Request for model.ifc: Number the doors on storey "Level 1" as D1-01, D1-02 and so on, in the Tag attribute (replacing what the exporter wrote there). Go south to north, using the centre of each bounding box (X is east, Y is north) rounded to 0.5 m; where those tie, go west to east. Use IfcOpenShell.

First a look at what the model holds.

```python
import ifcopenshell
import ifcopenshell.util.element
import ifcopenshell.util.placement

model = ifcopenshell.open("model.ifc")
print(model.schema)
storey = next(s for s in model.by_type("IfcBuildingStorey") if s.Name == "Level 1")
doors = [e for e in ifcopenshell.util.element.get_decomposition(storey) if e.is_a("IfcDoor")]
for e in sorted(doors, key=lambda e: e.id()):
    origin = ifcopenshell.util.placement.get_local_placement(e.ObjectPlacement)[:3, 3]
    print(e.id(), e.Tag, e.Name, origin.round(2) + 0.0, sep=" | ")
```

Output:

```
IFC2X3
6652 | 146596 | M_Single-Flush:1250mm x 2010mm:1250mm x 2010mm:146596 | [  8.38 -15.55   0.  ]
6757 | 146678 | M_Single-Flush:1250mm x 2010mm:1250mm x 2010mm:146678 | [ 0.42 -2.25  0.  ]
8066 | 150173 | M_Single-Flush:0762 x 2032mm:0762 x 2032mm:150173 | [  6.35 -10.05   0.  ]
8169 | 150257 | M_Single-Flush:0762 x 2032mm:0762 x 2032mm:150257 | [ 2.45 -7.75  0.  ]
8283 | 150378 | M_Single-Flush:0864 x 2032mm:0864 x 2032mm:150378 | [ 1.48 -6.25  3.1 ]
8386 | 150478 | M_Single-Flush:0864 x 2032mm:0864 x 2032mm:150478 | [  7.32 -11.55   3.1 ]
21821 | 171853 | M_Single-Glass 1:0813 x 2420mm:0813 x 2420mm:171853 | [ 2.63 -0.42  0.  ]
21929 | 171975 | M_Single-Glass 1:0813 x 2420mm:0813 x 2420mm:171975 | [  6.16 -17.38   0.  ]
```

```python
import ifcopenshell
import ifcopenshell.geom
import ifcopenshell.util.element
import ifcopenshell.util.shape

model = ifcopenshell.open("model.ifc")
settings = ifcopenshell.geom.settings()
settings.set("use-world-coords", True)


def centre(element):
    shape = ifcopenshell.geom.create_shape(settings, element)
    return ifcopenshell.util.shape.get_bbox_centroid(shape.geometry)


storey = next(s for s in model.by_type("IfcBuildingStorey") if s.Name == "Level 1")
doors = [e for e in ifcopenshell.util.element.get_decomposition(storey) if e.is_a("IfcDoor")]

# Insertion points can sit at a corner or the storey origin, so sort by the geometry (in metres).
centres = {e: centre(e) for e in doors}
doors.sort(key=lambda e: (round(centres[e][1] / 0.5), centres[e][0]))

for i, e in enumerate(doors, start=1):
    number = f"D1-{i:02d}"
    e.Tag = number
    print(e.id(), number)

model.write("model_rev.ifc")
```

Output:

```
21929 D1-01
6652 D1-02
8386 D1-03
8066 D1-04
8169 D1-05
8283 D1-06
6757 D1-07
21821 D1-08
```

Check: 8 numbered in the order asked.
